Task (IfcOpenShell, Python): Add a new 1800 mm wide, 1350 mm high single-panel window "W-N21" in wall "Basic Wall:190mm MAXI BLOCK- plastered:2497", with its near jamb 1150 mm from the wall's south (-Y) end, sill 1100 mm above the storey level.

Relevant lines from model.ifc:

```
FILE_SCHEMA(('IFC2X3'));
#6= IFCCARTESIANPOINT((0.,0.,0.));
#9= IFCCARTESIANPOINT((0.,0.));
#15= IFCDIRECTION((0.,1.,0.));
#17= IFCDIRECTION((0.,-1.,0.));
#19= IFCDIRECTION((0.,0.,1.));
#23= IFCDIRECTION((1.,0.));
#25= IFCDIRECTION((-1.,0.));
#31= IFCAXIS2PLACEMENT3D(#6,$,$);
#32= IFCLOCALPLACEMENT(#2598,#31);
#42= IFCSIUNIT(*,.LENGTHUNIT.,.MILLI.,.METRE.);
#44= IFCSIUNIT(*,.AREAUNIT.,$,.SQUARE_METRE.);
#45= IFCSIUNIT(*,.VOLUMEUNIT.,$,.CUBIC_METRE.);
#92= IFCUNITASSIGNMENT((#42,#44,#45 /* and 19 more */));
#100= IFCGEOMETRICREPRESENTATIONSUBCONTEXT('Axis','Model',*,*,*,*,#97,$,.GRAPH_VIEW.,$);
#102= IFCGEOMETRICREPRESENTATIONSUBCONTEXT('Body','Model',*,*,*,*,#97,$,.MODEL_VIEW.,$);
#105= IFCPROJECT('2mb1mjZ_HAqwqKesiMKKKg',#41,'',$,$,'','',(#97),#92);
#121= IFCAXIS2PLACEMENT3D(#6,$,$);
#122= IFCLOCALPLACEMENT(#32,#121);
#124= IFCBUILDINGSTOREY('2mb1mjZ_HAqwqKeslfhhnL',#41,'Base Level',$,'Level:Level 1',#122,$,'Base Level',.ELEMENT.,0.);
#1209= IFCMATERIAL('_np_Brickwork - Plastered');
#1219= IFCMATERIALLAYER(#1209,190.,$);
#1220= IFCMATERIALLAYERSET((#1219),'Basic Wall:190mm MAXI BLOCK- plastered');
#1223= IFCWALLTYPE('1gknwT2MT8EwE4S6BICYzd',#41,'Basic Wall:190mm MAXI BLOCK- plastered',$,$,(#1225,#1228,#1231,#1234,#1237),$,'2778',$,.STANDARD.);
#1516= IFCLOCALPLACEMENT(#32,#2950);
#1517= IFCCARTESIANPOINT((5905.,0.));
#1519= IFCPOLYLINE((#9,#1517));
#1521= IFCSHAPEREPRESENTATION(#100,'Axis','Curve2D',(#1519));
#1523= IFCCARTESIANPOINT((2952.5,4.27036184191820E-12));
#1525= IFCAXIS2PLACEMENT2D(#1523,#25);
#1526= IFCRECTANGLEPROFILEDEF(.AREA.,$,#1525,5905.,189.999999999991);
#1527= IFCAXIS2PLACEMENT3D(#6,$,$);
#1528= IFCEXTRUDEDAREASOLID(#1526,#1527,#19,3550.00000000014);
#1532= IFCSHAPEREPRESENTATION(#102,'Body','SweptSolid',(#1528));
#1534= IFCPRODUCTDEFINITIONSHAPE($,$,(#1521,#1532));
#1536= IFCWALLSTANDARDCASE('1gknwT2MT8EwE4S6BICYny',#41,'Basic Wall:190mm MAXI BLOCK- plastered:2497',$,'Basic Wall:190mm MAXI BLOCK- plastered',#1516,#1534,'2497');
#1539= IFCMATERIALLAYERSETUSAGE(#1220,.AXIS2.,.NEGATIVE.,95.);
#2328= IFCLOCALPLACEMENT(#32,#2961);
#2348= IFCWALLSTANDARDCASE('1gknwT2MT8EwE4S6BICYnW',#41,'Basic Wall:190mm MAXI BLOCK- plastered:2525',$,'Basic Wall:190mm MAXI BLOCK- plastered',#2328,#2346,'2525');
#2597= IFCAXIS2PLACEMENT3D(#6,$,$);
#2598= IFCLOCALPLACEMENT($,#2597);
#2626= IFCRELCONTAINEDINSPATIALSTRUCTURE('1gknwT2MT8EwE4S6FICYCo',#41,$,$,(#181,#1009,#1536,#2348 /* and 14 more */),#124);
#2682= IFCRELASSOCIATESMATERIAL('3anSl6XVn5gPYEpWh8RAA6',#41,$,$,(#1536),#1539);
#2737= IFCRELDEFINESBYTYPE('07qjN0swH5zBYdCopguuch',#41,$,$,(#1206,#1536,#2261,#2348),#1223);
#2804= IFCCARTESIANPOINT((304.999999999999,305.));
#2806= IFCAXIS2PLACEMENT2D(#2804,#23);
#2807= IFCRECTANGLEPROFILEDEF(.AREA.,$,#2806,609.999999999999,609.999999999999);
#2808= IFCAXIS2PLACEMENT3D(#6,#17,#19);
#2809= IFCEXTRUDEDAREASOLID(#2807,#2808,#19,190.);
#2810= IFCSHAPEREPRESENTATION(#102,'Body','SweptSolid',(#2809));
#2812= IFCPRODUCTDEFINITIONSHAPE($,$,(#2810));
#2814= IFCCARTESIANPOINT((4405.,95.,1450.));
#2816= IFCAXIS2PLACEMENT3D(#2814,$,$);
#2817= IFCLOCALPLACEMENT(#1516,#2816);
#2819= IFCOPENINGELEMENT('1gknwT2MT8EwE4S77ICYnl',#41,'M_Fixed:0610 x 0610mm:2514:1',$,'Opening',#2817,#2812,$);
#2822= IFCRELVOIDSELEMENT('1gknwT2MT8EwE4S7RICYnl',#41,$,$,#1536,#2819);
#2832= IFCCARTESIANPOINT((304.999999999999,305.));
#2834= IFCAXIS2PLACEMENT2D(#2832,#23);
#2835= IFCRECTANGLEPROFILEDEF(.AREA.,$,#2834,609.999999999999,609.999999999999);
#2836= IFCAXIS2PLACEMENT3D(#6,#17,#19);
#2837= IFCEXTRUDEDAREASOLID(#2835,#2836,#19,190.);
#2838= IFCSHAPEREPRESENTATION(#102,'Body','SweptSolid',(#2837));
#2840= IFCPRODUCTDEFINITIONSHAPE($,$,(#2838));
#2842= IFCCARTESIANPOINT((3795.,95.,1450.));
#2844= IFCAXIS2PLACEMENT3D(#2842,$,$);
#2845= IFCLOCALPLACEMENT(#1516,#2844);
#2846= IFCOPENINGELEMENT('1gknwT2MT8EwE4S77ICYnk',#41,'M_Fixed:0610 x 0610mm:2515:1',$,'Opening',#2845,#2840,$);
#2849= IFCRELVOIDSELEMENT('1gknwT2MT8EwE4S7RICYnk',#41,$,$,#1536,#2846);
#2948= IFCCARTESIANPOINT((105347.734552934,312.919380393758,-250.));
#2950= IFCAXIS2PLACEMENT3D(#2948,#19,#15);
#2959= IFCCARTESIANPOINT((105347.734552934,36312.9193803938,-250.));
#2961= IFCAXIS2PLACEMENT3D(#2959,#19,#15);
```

```python
import numpy as np
import ifcopenshell
import ifcopenshell.api.feature
import ifcopenshell.api.geometry
import ifcopenshell.api.root
import ifcopenshell.api.spatial
import ifcopenshell.api.type
import ifcopenshell.geom
import ifcopenshell.util.element
import ifcopenshell.util.placement
import ifcopenshell.util.representation
import ifcopenshell.util.shape
import ifcopenshell.util.unit

model = ifcopenshell.open("model.ifc")
unit_scale = ifcopenshell.util.unit.calculate_unit_scale(model)
settings = ifcopenshell.geom.settings()


def volume(element):
    """Net volume in cubic metres, openings subtracted."""
    shape = ifcopenshell.geom.create_shape(settings, element)
    return ifcopenshell.util.shape.get_volume(shape.geometry)


wall = model.by_guid("1gknwT2MT8EwE4S6BICYny")
storey = ifcopenshell.util.element.get_container(wall, ifc_class="IfcBuildingStorey")
context = ifcopenshell.util.representation.get_context(model, "Model", "Body", "MODEL_VIEW")
before = volume(wall)

width, height, from_end, sill = 1.8, 1.35, 1.15, 1.1  # metres

# The wall runs along its own X axis, and the end named is its -X end.
wall_shape = ifcopenshell.geom.create_shape(settings, wall)
x, y, z = ifcopenshell.util.shape.get_vertices(wall_shape.geometry).T
start = x.min() + from_end
face, thickness = float(y.min()), float(y.max() - y.min())
wall_matrix = ifcopenshell.util.placement.get_local_placement(wall.ObjectPlacement)
level = ifcopenshell.util.placement.get_local_placement(storey.ObjectPlacement)[2, 3]


def in_wall(x, y):
    """Placement at x, y metres in the wall's axes, at sill height."""
    matrix = wall_matrix.copy()
    matrix[:, 3] = wall_matrix @ np.array([x / unit_scale, y / unit_scale, 0.0, 1.0])
    matrix[2, 3] = level + sill / unit_scale
    return matrix


# Opening: a box that overshoots both wall faces by 50 mm.
opening = ifcopenshell.api.root.create_entity(model, ifc_class="IfcOpeningElement")
box = ifcopenshell.api.geometry.add_wall_representation(
    model, context=context, length=width, height=height, thickness=thickness + 0.1
)
ifcopenshell.api.geometry.assign_representation(model, product=opening, representation=box)
ifcopenshell.api.geometry.edit_object_placement(model, product=opening, matrix=in_wall(start, face - 0.05), is_si=False)
ifcopenshell.api.feature.add_feature(model, feature=opening, element=wall)

window = ifcopenshell.api.root.create_entity(model, ifc_class="IfcWindow", name="W-N21")
window.OverallWidth, window.OverallHeight = width / unit_scale, height / unit_scale
body = ifcopenshell.api.geometry.add_window_representation(
    model,
    context=context,
    overall_width=window.OverallWidth,
    overall_height=window.OverallHeight,
    partition_type="SINGLE_PANEL",
)
ifcopenshell.api.geometry.assign_representation(model, product=window, representation=body)
ifcopenshell.api.spatial.assign_container(model, products=[window], relating_structure=storey)
fills = ifcopenshell.api.feature.add_filling(model, opening=opening, element=window)
fills.OwnerHistory = window.OwnerHistory  # required in IFC2X3

# IFC2X3 keeps the operation on the window style.
style = ifcopenshell.api.root.create_entity(model, ifc_class="IfcWindowStyle", name="W-N21")
style.OperationType, style.ConstructionType = "SINGLE_PANEL", "NOTDEFINED"
style.ParameterTakesPrecedence = style.Sizeable = False
ifcopenshell.api.type.assign_type(model, related_objects=[window], relating_type=style)

# Centre the window in the wall's thickness.
ifcopenshell.api.geometry.edit_object_placement(model, product=window, matrix=in_wall(start, face), is_si=False)
window_shape = ifcopenshell.geom.create_shape(settings, window)
depth = ifcopenshell.util.shape.get_vertices(window_shape.geometry)[:, 1]
offset = face + thickness / 2 - (depth.min() + depth.max()) / 2
ifcopenshell.api.geometry.edit_object_placement(model, product=window, matrix=in_wall(start, offset), is_si=False)

after = volume(wall)

print(f"wall volume {before:.3f} -> {after:.3f} m3")

model.write("model_edited.ifc")
```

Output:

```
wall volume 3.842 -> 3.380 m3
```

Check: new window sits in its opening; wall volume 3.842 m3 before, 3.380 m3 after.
